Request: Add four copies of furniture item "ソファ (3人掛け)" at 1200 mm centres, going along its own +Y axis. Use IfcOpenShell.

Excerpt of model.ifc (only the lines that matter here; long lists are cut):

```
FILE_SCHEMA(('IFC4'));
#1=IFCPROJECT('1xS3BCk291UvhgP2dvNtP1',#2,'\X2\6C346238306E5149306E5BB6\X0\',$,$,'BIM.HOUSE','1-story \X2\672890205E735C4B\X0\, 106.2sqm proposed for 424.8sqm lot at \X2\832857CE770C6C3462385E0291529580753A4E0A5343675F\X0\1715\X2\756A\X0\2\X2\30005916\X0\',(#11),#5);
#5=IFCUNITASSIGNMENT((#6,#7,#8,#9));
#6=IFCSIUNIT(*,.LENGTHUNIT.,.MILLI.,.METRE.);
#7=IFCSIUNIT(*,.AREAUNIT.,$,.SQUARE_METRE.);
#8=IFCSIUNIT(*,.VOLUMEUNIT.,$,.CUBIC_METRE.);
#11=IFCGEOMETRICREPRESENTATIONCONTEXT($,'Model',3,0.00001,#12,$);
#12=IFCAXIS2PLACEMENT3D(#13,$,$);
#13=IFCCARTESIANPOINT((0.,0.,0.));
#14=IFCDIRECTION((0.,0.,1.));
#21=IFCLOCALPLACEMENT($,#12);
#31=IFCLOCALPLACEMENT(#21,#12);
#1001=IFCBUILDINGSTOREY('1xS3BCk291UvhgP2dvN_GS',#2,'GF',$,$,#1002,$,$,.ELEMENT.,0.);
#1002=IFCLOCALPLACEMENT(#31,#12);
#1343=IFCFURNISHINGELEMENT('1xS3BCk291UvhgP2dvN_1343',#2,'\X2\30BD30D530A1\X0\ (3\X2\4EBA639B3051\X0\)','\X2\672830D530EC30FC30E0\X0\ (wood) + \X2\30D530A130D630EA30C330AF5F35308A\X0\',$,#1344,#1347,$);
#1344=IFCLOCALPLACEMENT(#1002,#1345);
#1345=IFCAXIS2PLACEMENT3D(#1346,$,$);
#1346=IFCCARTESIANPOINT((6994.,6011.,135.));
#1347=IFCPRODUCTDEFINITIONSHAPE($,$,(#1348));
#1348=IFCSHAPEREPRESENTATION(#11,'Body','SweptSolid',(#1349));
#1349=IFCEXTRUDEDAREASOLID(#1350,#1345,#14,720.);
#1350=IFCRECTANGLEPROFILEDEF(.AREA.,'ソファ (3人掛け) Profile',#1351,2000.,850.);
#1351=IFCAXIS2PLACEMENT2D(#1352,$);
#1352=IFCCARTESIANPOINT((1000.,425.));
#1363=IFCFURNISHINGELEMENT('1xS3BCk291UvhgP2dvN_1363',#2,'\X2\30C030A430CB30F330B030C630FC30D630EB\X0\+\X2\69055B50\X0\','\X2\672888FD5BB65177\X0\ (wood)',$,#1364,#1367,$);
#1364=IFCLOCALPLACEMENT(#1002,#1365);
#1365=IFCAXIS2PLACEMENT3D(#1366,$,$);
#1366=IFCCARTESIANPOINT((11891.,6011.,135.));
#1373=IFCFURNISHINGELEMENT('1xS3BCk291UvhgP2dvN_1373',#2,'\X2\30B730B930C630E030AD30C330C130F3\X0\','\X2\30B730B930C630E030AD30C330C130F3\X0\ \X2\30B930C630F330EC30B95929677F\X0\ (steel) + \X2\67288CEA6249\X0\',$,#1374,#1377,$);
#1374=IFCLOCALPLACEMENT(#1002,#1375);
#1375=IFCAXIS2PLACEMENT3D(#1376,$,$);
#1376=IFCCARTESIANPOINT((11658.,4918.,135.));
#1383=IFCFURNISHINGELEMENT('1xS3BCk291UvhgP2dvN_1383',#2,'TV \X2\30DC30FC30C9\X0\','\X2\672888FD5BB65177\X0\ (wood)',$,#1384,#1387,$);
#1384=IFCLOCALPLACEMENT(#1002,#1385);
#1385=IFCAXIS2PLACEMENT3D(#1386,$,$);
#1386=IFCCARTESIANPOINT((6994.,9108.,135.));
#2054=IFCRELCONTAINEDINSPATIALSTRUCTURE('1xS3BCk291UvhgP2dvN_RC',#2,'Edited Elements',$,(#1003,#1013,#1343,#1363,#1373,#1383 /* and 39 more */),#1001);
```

```python
import ifcopenshell
import ifcopenshell.api.geometry
import ifcopenshell.api.root
import ifcopenshell.util.element
import ifcopenshell.util.placement
import ifcopenshell.util.unit

model = ifcopenshell.open("model.ifc")
unit_scale = ifcopenshell.util.unit.calculate_unit_scale(model)


def reuse_history(source, copy):
    """copy_class also copies each property set's owner history, people and application; keep the originals."""
    for rel in copy.IsDefinedBy:
        if rel.is_a("IfcRelDefinesByProperties") and (history := rel.RelatingPropertyDefinition.OwnerHistory):
            rel.RelatingPropertyDefinition.OwnerHistory = source.OwnerHistory
            ifcopenshell.util.element.remove_deep2(model, history)


source = model.by_guid("1xS3BCk291UvhgP2dvN_1343")
base = ifcopenshell.util.placement.get_local_placement(source.ObjectPlacement)
step = base[:3, 1] * 1.2 / unit_scale

for i in range(1, 5):
    copy = ifcopenshell.api.root.copy_class(model, product=source)
    copy.Representation = ifcopenshell.util.element.copy_deep(
        model, source.Representation, exclude=["IfcGeometricRepresentationContext", "IfcRepresentationMap"]
    )
    reuse_history(source, copy)
    matrix = base.copy()
    matrix[:3, 3] += i * step
    print("added at", matrix[:3, 3].round(3) + 0.0)
    ifcopenshell.api.geometry.edit_object_placement(model, product=copy, matrix=matrix, is_si=False)

model.write("model-out.ifc")
```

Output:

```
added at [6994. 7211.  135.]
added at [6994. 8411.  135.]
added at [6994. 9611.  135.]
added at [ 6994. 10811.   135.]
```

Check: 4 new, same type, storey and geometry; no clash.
